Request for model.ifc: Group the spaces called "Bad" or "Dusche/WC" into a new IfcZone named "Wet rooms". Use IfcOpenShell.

First a look at what the model holds.

```python
import ifcopenshell

model = ifcopenshell.open("model.ifc")
print(model.schema)
seen = {}
for space in model.by_type("IfcSpace"):
    seen[space.LongName] = seen.get(space.LongName, 0) + 1
for name, count in sorted(seen.items(), key=str):
    print(count, "x", name)
print("zones:", [z.Name for z in model.by_type("IfcZone")][:20])
```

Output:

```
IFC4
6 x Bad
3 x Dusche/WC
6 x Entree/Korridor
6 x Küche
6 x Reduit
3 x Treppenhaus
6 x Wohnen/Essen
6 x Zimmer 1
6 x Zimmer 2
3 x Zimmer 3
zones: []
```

```python
import ifcopenshell
import ifcopenshell.api.group
import ifcopenshell.api.root

model = ifcopenshell.open("model.ifc")

names = {"Bad", "Dusche/WC"}
spaces = [s for s in model.by_type("IfcSpace") if s.LongName in names]

zone = ifcopenshell.api.root.create_entity(model, ifc_class="IfcZone", name="Wet rooms")
ifcopenshell.api.group.assign_group(model, products=spaces, group=zone)
print(len(spaces), "spaces in", zone.Name)

model.write("model_updated.ifc")
```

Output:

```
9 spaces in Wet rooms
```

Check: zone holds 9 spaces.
